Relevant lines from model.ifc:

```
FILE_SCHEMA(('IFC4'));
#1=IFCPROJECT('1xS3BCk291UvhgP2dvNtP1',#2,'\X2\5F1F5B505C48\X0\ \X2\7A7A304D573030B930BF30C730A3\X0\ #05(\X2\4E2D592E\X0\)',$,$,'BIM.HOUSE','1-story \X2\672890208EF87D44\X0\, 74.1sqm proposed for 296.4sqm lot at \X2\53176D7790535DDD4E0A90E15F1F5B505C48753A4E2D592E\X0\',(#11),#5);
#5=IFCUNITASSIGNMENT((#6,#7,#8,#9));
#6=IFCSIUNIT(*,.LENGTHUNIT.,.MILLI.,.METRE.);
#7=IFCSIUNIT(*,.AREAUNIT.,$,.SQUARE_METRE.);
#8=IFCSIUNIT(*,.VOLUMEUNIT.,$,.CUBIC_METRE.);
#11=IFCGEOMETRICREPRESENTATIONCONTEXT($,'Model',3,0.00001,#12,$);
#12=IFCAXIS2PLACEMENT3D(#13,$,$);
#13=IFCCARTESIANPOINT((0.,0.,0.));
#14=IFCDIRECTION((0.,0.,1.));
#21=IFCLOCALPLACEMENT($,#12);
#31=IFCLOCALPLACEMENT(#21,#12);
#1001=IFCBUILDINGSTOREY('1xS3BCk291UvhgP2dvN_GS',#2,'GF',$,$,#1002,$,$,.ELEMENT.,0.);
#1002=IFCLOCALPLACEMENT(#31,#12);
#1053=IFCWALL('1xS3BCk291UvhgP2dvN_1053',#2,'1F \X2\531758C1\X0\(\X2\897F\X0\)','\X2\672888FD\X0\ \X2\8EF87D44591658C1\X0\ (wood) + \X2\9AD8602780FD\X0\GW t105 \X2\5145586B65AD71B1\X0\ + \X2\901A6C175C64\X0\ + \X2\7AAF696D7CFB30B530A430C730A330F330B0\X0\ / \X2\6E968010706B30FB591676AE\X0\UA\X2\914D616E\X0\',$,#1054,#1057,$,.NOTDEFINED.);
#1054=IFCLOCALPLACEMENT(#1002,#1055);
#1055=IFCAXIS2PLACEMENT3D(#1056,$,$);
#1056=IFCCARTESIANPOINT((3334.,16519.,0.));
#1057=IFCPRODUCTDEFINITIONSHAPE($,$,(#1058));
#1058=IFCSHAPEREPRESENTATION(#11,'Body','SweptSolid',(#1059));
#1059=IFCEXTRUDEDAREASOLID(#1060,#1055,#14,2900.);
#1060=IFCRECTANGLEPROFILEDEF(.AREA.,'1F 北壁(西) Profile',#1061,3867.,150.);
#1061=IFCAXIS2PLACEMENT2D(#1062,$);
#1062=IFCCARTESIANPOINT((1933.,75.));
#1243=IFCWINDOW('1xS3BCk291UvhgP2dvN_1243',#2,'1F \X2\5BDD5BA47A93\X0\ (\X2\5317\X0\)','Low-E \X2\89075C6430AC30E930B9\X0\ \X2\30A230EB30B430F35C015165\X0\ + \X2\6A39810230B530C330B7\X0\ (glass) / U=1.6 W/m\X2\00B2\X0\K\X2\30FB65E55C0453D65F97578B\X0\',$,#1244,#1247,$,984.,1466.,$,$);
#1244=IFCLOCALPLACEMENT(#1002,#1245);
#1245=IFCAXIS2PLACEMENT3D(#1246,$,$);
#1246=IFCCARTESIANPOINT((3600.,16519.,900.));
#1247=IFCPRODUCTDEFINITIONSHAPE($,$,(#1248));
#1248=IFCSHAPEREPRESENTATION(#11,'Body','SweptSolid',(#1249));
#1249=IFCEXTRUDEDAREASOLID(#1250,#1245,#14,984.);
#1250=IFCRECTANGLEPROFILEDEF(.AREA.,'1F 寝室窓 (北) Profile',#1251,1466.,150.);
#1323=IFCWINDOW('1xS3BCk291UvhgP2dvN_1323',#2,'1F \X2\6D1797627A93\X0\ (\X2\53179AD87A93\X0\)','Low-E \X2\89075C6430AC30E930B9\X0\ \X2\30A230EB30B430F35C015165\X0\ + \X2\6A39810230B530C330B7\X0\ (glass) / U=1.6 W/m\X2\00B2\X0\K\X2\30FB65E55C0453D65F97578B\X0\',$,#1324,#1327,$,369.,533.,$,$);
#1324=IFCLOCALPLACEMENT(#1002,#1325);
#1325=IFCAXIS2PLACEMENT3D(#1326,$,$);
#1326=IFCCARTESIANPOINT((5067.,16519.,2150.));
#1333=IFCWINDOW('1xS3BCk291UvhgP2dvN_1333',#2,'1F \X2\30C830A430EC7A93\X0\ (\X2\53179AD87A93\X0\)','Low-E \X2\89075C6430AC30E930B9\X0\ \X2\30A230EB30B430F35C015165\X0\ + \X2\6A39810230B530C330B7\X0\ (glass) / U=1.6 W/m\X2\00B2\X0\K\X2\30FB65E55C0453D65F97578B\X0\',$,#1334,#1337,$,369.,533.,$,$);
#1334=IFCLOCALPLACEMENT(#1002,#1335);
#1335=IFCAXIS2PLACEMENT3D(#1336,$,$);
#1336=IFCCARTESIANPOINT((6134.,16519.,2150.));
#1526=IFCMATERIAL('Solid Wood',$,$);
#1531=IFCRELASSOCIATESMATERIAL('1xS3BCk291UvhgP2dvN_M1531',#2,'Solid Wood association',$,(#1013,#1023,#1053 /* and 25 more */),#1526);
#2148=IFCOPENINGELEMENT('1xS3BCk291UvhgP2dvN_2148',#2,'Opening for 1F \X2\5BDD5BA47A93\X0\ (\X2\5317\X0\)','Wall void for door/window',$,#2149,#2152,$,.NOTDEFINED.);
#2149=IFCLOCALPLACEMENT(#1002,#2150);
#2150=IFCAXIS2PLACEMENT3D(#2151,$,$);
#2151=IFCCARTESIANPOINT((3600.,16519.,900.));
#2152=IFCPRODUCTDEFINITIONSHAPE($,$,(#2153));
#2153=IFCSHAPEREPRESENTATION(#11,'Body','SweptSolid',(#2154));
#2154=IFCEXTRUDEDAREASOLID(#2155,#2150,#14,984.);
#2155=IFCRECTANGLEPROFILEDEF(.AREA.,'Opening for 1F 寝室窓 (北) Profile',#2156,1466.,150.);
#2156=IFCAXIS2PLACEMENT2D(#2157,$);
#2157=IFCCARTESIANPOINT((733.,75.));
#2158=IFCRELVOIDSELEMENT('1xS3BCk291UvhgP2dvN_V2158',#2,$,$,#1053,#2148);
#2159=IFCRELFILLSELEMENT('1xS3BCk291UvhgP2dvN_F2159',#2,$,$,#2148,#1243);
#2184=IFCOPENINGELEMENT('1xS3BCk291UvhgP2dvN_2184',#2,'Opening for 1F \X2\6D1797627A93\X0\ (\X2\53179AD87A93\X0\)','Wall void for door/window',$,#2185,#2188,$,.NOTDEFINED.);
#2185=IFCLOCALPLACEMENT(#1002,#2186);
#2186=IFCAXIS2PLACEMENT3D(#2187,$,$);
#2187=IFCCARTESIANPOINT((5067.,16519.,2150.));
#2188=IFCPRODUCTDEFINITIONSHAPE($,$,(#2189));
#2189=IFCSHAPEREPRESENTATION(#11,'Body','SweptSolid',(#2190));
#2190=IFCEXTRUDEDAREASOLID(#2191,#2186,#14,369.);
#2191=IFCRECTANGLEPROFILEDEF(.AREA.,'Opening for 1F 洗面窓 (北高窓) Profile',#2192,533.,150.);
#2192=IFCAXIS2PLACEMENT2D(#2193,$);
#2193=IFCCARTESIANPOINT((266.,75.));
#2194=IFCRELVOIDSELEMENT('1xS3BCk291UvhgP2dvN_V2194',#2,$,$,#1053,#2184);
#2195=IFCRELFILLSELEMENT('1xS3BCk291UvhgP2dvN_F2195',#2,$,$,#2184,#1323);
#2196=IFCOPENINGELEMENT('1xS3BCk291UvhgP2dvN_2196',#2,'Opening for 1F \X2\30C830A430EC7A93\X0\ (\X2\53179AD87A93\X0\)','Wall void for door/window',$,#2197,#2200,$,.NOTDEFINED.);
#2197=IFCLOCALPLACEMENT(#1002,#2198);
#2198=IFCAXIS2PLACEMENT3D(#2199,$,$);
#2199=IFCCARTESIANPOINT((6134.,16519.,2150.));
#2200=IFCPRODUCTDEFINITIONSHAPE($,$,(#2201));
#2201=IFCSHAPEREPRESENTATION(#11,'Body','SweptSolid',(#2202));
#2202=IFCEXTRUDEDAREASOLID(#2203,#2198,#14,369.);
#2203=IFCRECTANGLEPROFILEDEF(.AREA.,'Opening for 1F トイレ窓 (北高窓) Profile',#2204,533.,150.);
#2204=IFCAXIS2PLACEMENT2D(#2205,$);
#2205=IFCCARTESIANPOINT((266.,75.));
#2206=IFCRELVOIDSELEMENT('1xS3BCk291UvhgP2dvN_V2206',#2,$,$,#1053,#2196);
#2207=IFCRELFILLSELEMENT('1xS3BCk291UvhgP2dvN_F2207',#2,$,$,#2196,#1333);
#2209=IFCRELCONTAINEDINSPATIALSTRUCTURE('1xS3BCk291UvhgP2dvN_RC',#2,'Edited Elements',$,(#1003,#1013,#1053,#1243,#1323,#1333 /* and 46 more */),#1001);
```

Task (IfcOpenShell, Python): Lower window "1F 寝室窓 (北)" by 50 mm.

```python
import numpy as np
import ifcopenshell
import ifcopenshell.api.geometry
import ifcopenshell.util.placement
import ifcopenshell.util.unit

model = ifcopenshell.open("model.ifc")
unit_scale = ifcopenshell.util.unit.calculate_unit_scale(model)

window = model.by_guid("1xS3BCk291UvhgP2dvN_1243")
opening = window.FillsVoids[0].RelatingOpeningElement
dz = -50.0

shift = np.array([0.0, 0.0, dz])
# The window is not placed relative to its opening, so move both.
for product in (opening, window):
    matrix = ifcopenshell.util.placement.get_local_placement(product.ObjectPlacement)
    matrix[:3, 3] += shift
    ifcopenshell.api.geometry.edit_object_placement(model, product=product, matrix=matrix, is_si=False)

print(f"moved by {dz * unit_scale:+.3f} m")

model.write("model_updated.ifc")
```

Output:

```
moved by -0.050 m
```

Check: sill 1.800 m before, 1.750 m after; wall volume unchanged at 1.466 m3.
